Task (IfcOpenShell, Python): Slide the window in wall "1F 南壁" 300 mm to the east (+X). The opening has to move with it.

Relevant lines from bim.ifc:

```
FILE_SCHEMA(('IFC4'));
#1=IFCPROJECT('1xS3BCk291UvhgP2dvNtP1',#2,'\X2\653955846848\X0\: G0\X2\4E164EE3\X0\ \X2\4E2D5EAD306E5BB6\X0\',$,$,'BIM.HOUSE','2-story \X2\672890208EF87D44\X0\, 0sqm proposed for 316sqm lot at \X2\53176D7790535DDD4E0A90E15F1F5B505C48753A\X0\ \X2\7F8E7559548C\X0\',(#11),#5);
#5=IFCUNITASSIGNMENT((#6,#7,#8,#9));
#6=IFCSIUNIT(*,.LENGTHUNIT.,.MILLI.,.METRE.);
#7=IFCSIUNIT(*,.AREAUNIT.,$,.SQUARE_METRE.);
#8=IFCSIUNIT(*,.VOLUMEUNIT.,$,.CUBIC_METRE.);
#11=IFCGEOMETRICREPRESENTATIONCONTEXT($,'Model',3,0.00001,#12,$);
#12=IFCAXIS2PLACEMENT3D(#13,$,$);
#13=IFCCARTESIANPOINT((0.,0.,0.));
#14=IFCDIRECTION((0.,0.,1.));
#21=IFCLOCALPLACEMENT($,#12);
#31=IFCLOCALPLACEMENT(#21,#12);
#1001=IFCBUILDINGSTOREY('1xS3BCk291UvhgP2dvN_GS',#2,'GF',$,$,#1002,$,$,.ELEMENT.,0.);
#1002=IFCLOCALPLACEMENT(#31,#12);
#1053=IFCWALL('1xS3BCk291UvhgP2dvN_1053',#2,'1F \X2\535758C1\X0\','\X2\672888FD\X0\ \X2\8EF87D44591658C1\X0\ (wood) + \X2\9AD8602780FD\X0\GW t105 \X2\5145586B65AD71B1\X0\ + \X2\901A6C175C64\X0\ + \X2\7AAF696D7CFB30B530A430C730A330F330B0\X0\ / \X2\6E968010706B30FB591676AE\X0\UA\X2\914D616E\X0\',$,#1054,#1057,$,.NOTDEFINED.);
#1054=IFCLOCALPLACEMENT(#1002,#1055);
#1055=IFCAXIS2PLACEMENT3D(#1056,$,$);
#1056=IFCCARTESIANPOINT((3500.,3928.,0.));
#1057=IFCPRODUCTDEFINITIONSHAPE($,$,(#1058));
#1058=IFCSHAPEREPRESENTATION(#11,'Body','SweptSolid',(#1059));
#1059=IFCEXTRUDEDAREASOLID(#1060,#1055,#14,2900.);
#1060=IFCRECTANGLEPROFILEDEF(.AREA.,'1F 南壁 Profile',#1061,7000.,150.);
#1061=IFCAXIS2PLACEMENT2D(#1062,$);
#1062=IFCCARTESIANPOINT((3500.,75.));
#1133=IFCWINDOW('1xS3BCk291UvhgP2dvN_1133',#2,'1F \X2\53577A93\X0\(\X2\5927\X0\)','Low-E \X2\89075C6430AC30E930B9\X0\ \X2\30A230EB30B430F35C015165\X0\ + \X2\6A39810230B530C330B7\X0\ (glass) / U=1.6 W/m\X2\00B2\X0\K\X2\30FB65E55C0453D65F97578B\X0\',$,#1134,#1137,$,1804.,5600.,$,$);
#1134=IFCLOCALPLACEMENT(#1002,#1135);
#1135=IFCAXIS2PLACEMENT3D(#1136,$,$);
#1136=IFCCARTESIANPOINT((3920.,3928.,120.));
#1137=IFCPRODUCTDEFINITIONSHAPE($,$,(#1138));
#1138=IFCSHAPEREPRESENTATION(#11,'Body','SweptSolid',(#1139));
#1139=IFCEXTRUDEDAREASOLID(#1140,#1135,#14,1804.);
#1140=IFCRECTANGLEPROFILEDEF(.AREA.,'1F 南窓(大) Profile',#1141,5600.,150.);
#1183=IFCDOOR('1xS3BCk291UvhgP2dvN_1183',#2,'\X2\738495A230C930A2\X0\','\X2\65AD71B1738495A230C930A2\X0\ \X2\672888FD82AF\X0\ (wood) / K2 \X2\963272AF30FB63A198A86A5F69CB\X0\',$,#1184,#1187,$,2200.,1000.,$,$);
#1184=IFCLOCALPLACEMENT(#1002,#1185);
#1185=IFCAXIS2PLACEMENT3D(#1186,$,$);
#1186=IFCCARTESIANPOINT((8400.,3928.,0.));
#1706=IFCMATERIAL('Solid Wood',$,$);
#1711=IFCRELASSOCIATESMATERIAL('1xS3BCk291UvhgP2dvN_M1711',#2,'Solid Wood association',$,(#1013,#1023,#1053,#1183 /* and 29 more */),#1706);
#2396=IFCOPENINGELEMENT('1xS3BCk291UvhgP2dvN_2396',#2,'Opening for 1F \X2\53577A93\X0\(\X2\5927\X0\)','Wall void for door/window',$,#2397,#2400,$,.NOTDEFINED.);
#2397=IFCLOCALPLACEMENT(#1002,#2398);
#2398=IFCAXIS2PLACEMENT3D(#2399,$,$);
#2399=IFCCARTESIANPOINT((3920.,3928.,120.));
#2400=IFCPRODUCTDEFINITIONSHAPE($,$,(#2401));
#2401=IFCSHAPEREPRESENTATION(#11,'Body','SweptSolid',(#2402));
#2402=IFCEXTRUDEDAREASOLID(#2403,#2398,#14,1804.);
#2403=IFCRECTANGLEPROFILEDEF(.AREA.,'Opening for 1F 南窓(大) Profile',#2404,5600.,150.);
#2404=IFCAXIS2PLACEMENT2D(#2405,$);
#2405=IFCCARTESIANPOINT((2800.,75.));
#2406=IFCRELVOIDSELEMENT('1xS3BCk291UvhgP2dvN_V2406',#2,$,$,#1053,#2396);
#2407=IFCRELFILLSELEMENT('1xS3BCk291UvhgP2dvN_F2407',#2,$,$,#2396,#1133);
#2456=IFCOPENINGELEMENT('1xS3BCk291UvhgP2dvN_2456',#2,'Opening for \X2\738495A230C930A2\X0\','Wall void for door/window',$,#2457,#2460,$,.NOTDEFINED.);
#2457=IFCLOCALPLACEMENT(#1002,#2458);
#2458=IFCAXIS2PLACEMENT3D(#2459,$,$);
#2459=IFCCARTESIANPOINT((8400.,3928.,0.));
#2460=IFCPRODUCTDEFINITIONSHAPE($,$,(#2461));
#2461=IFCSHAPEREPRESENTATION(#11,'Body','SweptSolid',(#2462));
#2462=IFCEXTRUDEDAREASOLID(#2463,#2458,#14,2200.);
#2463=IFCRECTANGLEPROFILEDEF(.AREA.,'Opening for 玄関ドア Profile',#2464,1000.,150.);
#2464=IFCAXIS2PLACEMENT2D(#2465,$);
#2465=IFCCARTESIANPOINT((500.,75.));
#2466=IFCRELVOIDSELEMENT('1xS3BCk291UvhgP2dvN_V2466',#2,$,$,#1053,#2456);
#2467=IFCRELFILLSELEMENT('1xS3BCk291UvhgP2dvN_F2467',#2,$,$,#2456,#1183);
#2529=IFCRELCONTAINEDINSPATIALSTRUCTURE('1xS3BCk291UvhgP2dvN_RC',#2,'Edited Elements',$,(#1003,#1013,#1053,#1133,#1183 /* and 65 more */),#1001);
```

```python
import ifcopenshell
import ifcopenshell.api.geometry
import ifcopenshell.util.placement

model = ifcopenshell.open("bim.ifc")

window = model.by_guid("1xS3BCk291UvhgP2dvN_1133")
opening = window.FillsVoids[0].RelatingOpeningElement
wall = opening.VoidsElements[0].RelatingBuildingElement

wall_matrix = ifcopenshell.util.placement.get_local_placement(wall.ObjectPlacement)
shift = wall_matrix[:3, 0] * 300.0
before = ifcopenshell.util.placement.get_local_placement(window.ObjectPlacement)[:3, 3].copy()

# The window is not placed relative to its opening, so move both.
for product in (opening, window):
    matrix = ifcopenshell.util.placement.get_local_placement(product.ObjectPlacement)
    matrix[:3, 3] += shift
    ifcopenshell.api.geometry.edit_object_placement(model, product=product, matrix=matrix, is_si=False)

after = ifcopenshell.util.placement.get_local_placement(window.ObjectPlacement)[:3, 3]
print("window moved by", (after - before).round(3) + 0.0)

model.write("bim_updated.ifc")
```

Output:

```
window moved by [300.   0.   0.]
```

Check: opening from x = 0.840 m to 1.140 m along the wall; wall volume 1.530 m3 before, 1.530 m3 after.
